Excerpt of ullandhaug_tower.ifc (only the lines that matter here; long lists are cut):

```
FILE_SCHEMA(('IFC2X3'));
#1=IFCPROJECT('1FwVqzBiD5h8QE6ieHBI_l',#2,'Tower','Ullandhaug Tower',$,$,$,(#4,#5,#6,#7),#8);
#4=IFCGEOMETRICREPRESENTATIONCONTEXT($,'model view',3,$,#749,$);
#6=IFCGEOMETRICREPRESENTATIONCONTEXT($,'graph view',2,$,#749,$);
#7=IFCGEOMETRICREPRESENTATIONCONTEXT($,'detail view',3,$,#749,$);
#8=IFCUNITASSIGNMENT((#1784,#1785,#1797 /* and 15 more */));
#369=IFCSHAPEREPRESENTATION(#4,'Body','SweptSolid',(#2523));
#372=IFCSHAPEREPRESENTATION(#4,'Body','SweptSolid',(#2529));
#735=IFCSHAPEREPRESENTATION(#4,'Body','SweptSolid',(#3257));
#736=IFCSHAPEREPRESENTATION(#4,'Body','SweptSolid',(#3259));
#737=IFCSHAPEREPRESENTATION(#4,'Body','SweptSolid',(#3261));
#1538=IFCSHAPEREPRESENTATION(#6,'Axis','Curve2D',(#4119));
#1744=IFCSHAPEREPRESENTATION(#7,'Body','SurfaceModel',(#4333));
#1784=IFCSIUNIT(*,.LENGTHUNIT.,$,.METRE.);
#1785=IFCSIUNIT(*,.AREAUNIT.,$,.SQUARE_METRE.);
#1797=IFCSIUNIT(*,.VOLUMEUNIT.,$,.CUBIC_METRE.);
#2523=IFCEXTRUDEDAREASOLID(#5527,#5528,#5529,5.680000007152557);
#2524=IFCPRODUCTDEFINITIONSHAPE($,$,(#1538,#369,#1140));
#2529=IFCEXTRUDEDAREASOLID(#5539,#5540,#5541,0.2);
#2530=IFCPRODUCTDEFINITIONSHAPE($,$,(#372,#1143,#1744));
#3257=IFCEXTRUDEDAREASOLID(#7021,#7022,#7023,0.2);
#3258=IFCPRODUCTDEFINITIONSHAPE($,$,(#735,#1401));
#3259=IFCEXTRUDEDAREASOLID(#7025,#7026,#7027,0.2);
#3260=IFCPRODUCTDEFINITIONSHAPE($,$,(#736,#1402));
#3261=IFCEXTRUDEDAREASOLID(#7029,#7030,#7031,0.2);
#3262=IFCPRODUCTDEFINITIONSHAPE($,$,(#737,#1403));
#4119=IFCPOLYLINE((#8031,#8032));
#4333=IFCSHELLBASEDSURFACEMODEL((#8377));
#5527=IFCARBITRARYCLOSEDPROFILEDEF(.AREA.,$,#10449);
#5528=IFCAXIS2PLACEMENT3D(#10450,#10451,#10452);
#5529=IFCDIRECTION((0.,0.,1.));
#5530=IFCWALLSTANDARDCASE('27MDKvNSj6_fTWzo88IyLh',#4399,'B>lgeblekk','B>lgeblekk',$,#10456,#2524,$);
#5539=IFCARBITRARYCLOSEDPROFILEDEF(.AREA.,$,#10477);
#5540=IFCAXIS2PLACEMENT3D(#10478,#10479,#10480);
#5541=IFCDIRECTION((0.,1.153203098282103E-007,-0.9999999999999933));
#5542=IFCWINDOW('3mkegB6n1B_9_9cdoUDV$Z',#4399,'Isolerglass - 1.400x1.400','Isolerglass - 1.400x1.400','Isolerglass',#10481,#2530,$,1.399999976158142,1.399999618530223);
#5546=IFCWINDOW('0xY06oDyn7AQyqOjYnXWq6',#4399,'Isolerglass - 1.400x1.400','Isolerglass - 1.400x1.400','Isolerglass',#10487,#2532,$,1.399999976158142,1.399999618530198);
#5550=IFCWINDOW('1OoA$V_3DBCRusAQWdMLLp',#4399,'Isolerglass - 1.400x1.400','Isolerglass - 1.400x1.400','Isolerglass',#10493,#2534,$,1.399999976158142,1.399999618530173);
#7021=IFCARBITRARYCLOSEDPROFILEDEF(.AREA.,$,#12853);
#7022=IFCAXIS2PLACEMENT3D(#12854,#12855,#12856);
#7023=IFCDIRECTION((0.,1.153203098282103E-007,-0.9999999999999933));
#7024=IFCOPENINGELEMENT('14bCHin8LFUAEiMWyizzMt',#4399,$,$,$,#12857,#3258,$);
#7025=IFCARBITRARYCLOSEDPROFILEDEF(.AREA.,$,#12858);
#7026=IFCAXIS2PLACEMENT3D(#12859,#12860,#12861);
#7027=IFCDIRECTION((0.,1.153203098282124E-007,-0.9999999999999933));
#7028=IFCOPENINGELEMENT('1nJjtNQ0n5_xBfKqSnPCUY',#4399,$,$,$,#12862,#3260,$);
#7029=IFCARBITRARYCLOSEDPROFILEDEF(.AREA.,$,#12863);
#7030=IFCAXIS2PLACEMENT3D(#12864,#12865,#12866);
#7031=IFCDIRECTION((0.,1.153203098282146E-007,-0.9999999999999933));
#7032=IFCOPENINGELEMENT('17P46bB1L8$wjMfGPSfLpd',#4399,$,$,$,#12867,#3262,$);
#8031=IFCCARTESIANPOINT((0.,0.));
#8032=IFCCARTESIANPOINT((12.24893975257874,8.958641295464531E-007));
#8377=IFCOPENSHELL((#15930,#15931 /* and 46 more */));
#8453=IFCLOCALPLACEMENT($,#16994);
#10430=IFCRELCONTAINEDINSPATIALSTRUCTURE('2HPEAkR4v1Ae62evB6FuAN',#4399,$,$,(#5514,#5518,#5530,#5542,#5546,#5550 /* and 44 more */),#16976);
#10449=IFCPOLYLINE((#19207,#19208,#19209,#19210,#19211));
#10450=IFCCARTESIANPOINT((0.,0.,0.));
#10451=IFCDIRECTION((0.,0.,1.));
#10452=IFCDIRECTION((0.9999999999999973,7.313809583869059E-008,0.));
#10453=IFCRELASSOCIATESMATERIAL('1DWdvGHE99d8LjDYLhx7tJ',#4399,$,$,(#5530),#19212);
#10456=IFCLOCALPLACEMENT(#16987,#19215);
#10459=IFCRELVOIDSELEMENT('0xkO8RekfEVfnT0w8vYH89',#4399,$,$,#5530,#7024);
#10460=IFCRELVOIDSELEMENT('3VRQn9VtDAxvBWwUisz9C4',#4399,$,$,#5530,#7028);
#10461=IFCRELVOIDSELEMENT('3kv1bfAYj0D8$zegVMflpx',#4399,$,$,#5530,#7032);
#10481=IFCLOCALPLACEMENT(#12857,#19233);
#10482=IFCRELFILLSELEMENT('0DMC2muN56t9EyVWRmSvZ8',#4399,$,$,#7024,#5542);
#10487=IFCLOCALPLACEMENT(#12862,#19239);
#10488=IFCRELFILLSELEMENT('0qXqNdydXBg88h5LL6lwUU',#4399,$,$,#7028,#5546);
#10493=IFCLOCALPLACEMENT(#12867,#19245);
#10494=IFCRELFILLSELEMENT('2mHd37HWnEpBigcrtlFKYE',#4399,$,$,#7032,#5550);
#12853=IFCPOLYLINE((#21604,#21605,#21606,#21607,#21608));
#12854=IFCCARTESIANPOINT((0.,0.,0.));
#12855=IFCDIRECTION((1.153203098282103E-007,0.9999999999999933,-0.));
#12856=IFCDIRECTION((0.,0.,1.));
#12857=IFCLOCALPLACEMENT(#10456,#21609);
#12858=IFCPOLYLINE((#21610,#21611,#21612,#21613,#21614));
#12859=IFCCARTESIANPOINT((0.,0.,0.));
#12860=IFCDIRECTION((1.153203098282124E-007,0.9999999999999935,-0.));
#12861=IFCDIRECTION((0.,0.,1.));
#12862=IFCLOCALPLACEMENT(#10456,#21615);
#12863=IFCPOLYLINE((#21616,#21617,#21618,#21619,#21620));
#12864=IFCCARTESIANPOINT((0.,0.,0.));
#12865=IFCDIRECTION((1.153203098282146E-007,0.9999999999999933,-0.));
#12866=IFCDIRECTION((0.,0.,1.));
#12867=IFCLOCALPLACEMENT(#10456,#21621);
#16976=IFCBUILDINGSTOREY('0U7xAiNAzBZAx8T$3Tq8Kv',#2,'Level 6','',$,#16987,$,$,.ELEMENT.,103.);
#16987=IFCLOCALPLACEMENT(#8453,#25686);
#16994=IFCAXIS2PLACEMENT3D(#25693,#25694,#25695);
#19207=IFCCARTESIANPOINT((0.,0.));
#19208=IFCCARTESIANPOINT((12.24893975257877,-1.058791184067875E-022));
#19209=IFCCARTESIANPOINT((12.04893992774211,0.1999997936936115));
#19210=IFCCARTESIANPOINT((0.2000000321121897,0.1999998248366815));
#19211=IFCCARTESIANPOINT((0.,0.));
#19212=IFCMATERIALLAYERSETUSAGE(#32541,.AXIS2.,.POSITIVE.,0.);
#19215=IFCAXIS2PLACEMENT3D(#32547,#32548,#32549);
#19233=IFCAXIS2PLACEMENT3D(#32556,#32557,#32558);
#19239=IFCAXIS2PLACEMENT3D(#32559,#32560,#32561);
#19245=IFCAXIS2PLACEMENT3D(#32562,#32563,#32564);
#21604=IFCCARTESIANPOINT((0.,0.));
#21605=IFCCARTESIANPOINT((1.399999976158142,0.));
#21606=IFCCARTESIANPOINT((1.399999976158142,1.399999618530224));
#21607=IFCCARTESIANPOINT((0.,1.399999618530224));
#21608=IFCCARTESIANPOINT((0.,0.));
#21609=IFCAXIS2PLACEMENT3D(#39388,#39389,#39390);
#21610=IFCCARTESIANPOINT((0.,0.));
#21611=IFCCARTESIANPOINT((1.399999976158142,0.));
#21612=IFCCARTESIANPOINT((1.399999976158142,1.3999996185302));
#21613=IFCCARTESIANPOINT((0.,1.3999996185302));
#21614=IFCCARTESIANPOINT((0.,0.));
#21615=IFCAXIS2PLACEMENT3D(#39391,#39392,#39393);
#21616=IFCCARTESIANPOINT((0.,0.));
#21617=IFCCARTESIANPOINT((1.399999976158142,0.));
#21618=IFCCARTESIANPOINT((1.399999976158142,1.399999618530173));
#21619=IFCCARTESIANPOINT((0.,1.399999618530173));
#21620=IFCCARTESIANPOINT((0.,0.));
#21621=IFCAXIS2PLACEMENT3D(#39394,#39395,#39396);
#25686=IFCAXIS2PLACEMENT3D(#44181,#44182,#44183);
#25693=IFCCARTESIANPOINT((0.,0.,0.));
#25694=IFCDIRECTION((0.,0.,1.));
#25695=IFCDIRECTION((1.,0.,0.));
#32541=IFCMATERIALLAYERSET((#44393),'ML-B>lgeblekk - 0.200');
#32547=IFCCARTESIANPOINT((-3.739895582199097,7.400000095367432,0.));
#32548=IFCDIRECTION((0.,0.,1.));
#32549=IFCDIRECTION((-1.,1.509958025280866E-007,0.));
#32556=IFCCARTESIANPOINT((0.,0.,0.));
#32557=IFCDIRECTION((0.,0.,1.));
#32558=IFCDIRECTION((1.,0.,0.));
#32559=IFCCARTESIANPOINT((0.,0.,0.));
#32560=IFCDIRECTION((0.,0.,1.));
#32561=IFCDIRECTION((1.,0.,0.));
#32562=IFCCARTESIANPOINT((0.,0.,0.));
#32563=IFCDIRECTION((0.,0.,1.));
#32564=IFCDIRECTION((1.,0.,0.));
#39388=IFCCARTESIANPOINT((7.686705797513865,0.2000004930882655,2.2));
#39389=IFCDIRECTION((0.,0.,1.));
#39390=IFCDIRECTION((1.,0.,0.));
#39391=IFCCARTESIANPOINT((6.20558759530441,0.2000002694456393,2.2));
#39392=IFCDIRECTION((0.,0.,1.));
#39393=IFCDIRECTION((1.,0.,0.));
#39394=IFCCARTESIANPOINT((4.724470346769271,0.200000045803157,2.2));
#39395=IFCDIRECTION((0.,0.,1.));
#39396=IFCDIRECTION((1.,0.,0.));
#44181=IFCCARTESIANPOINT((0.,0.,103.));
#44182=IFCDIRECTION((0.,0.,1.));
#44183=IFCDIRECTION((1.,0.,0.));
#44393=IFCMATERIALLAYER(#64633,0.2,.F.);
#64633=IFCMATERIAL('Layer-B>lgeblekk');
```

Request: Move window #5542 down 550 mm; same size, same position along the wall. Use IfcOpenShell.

```python
import numpy as np
import ifcopenshell
import ifcopenshell.api.geometry
import ifcopenshell.util.placement
import ifcopenshell.util.unit

model = ifcopenshell.open("ullandhaug_tower.ifc")
unit_scale = ifcopenshell.util.unit.calculate_unit_scale(model)

window = model.by_id(5542)
opening = window.FillsVoids[0].RelatingOpeningElement
dz = -0.55 / unit_scale

shift = np.array([0.0, 0.0, dz])
# The window is placed relative to its opening, so it follows when the opening moves.
matrix = ifcopenshell.util.placement.get_local_placement(opening.ObjectPlacement)
matrix[:3, 3] += shift
ifcopenshell.api.geometry.edit_object_placement(
    model, product=opening, matrix=matrix, is_si=False, should_transform_children=True
)

print(f"moved by {dz * unit_scale:+.3f} m")

model.write("ullandhaug_tower_rev.ifc")
```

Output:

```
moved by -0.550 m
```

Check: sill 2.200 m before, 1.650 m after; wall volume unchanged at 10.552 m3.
